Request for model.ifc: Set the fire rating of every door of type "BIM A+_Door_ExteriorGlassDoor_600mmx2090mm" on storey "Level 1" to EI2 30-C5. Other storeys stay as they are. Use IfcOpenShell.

First a look at what the model holds.

```python
import ifcopenshell
import ifcopenshell.util.element

model = ifcopenshell.open("model.ifc")
print(model.schema)
storey = next(s for s in model.by_type("IfcBuildingStorey") if s.Name == "Level 1")
doors = [e for e in ifcopenshell.util.element.get_decomposition(storey) if e.is_a("IfcDoor")]
seen = {}
for e in doors:
    element_type = ifcopenshell.util.element.get_type(e)
    key = (element_type.Name if element_type != e and element_type else None, ifcopenshell.util.element.get_pset(e, "Pset_DoorCommon", "FireRating"))
    seen[key] = seen.get(key, 0) + 1
for (name, value), count in sorted(seen.items(), key=str):
    print(count, "x", name, "|", value)
```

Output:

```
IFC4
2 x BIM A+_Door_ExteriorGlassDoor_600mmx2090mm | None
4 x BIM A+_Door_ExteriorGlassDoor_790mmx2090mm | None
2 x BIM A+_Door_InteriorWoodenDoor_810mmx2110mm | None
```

```python
import ifcopenshell
import ifcopenshell.api.pset
import ifcopenshell.util.element

model = ifcopenshell.open("model.ifc")

storey = next(s for s in model.by_type("IfcBuildingStorey") if s.Name == "Level 1")
doors = [e for e in ifcopenshell.util.element.get_decomposition(storey) if e.is_a("IfcDoor")]

count = 0
for e in doors:
    element_type = ifcopenshell.util.element.get_type(e)
    if element_type in (None, e) or element_type.Name != "BIM A+_Door_ExteriorGlassDoor_600mmx2090mm":
        continue
    # add_pset returns the element's existing set when there is one.
    pset = ifcopenshell.api.pset.add_pset(model, product=e, name="Pset_DoorCommon")
    ifcopenshell.api.pset.edit_pset(model, pset=pset, properties={"FireRating": "EI2 30-C5"})
    count += 1

print(count, "doors updated")

model.write("model_updated.ifc")
```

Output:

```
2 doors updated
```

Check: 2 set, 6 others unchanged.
